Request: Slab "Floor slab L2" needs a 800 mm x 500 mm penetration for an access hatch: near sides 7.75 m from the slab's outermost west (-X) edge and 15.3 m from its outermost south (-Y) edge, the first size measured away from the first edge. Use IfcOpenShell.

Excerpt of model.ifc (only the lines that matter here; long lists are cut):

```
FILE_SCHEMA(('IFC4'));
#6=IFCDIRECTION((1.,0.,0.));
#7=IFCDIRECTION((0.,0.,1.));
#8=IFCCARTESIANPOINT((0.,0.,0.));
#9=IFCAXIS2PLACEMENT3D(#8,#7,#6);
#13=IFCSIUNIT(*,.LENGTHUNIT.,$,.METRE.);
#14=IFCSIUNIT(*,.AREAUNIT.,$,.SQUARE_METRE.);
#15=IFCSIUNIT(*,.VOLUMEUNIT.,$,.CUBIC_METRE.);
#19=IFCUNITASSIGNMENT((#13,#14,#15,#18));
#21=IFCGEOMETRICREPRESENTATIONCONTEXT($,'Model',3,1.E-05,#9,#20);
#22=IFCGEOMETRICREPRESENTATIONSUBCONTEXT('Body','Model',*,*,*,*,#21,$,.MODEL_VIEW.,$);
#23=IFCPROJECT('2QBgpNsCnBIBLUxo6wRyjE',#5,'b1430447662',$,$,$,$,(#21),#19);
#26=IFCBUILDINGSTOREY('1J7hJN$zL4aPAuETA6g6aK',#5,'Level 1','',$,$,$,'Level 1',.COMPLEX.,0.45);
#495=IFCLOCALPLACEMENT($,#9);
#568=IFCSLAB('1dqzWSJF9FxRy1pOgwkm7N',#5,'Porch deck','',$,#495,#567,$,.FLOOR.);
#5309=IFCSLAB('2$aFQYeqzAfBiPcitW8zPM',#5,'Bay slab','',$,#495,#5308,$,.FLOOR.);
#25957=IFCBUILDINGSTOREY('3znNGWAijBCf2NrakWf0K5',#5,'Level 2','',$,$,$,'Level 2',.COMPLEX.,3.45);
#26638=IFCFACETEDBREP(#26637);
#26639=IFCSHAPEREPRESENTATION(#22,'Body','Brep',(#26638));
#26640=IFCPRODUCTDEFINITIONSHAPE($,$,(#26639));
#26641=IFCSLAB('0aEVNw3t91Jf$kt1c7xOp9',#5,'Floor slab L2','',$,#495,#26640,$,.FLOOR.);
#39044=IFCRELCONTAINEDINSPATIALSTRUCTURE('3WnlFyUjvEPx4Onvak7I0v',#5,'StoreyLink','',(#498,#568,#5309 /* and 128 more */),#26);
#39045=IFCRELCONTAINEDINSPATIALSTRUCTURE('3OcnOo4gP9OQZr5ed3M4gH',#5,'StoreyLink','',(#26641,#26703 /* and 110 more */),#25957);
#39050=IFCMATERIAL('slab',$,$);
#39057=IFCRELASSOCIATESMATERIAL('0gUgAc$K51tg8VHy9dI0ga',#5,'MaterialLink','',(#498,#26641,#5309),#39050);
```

```python
import numpy as np
import ifcopenshell
import ifcopenshell.api.feature
import ifcopenshell.api.geometry
import ifcopenshell.api.root
import ifcopenshell.geom
import ifcopenshell.util.placement
import ifcopenshell.util.representation
import ifcopenshell.util.shape
import ifcopenshell.util.unit

model = ifcopenshell.open("model.ifc")
unit_scale = ifcopenshell.util.unit.calculate_unit_scale(model)
settings = ifcopenshell.geom.settings()


def volume(element):
    """Net volume in cubic metres, openings subtracted."""
    shape = ifcopenshell.geom.create_shape(settings, element)
    return ifcopenshell.util.shape.get_volume(shape.geometry)


slab = model.by_guid("0aEVNw3t91Jf$kt1c7xOp9")
before = volume(slab)

# Extent in the slab's own axes, in metres. The edges named are its -X and -Y sides.
slab_shape = ifcopenshell.geom.create_shape(settings, slab)
vertices = ifcopenshell.util.shape.get_vertices(slab_shape.geometry)
x_min, y_min, bottom = vertices.min(axis=0)
top = vertices[:, 2].max()

opening = ifcopenshell.api.root.create_entity(model, ifc_class="IfcOpeningElement", name="Access hatch opening", predefined_type="OPENING")
context = ifcopenshell.util.representation.get_context(model, "Model", "Body", "MODEL_VIEW")
width, depth = 0.8, 0.5
outline = [(0.0, 0.0), (width, 0.0), (width, depth), (0.0, depth), (0.0, 0.0)]
# Overshoot both faces by 50 mm so the cut is clean.
shape = ifcopenshell.api.geometry.add_slab_representation(
    model, context=context, depth=top - bottom + 0.1, polyline=outline
)
ifcopenshell.api.geometry.assign_representation(model, product=opening, representation=shape)

matrix = ifcopenshell.util.placement.get_local_placement(slab.ObjectPlacement)
matrix[:, 3] = matrix @ np.append(np.array([x_min + 7.75, y_min + 15.3, bottom - 0.05]) / unit_scale, 1.0)
ifcopenshell.api.geometry.edit_object_placement(model, product=opening, matrix=matrix, is_si=False)
ifcopenshell.api.feature.add_feature(model, feature=opening, element=slab)

after = volume(slab)

print(f"slab volume {before:.3f} -> {after:.3f} m3")

model.write("model_rev.ifc")
```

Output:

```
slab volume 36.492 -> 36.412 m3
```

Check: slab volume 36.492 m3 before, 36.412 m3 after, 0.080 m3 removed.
